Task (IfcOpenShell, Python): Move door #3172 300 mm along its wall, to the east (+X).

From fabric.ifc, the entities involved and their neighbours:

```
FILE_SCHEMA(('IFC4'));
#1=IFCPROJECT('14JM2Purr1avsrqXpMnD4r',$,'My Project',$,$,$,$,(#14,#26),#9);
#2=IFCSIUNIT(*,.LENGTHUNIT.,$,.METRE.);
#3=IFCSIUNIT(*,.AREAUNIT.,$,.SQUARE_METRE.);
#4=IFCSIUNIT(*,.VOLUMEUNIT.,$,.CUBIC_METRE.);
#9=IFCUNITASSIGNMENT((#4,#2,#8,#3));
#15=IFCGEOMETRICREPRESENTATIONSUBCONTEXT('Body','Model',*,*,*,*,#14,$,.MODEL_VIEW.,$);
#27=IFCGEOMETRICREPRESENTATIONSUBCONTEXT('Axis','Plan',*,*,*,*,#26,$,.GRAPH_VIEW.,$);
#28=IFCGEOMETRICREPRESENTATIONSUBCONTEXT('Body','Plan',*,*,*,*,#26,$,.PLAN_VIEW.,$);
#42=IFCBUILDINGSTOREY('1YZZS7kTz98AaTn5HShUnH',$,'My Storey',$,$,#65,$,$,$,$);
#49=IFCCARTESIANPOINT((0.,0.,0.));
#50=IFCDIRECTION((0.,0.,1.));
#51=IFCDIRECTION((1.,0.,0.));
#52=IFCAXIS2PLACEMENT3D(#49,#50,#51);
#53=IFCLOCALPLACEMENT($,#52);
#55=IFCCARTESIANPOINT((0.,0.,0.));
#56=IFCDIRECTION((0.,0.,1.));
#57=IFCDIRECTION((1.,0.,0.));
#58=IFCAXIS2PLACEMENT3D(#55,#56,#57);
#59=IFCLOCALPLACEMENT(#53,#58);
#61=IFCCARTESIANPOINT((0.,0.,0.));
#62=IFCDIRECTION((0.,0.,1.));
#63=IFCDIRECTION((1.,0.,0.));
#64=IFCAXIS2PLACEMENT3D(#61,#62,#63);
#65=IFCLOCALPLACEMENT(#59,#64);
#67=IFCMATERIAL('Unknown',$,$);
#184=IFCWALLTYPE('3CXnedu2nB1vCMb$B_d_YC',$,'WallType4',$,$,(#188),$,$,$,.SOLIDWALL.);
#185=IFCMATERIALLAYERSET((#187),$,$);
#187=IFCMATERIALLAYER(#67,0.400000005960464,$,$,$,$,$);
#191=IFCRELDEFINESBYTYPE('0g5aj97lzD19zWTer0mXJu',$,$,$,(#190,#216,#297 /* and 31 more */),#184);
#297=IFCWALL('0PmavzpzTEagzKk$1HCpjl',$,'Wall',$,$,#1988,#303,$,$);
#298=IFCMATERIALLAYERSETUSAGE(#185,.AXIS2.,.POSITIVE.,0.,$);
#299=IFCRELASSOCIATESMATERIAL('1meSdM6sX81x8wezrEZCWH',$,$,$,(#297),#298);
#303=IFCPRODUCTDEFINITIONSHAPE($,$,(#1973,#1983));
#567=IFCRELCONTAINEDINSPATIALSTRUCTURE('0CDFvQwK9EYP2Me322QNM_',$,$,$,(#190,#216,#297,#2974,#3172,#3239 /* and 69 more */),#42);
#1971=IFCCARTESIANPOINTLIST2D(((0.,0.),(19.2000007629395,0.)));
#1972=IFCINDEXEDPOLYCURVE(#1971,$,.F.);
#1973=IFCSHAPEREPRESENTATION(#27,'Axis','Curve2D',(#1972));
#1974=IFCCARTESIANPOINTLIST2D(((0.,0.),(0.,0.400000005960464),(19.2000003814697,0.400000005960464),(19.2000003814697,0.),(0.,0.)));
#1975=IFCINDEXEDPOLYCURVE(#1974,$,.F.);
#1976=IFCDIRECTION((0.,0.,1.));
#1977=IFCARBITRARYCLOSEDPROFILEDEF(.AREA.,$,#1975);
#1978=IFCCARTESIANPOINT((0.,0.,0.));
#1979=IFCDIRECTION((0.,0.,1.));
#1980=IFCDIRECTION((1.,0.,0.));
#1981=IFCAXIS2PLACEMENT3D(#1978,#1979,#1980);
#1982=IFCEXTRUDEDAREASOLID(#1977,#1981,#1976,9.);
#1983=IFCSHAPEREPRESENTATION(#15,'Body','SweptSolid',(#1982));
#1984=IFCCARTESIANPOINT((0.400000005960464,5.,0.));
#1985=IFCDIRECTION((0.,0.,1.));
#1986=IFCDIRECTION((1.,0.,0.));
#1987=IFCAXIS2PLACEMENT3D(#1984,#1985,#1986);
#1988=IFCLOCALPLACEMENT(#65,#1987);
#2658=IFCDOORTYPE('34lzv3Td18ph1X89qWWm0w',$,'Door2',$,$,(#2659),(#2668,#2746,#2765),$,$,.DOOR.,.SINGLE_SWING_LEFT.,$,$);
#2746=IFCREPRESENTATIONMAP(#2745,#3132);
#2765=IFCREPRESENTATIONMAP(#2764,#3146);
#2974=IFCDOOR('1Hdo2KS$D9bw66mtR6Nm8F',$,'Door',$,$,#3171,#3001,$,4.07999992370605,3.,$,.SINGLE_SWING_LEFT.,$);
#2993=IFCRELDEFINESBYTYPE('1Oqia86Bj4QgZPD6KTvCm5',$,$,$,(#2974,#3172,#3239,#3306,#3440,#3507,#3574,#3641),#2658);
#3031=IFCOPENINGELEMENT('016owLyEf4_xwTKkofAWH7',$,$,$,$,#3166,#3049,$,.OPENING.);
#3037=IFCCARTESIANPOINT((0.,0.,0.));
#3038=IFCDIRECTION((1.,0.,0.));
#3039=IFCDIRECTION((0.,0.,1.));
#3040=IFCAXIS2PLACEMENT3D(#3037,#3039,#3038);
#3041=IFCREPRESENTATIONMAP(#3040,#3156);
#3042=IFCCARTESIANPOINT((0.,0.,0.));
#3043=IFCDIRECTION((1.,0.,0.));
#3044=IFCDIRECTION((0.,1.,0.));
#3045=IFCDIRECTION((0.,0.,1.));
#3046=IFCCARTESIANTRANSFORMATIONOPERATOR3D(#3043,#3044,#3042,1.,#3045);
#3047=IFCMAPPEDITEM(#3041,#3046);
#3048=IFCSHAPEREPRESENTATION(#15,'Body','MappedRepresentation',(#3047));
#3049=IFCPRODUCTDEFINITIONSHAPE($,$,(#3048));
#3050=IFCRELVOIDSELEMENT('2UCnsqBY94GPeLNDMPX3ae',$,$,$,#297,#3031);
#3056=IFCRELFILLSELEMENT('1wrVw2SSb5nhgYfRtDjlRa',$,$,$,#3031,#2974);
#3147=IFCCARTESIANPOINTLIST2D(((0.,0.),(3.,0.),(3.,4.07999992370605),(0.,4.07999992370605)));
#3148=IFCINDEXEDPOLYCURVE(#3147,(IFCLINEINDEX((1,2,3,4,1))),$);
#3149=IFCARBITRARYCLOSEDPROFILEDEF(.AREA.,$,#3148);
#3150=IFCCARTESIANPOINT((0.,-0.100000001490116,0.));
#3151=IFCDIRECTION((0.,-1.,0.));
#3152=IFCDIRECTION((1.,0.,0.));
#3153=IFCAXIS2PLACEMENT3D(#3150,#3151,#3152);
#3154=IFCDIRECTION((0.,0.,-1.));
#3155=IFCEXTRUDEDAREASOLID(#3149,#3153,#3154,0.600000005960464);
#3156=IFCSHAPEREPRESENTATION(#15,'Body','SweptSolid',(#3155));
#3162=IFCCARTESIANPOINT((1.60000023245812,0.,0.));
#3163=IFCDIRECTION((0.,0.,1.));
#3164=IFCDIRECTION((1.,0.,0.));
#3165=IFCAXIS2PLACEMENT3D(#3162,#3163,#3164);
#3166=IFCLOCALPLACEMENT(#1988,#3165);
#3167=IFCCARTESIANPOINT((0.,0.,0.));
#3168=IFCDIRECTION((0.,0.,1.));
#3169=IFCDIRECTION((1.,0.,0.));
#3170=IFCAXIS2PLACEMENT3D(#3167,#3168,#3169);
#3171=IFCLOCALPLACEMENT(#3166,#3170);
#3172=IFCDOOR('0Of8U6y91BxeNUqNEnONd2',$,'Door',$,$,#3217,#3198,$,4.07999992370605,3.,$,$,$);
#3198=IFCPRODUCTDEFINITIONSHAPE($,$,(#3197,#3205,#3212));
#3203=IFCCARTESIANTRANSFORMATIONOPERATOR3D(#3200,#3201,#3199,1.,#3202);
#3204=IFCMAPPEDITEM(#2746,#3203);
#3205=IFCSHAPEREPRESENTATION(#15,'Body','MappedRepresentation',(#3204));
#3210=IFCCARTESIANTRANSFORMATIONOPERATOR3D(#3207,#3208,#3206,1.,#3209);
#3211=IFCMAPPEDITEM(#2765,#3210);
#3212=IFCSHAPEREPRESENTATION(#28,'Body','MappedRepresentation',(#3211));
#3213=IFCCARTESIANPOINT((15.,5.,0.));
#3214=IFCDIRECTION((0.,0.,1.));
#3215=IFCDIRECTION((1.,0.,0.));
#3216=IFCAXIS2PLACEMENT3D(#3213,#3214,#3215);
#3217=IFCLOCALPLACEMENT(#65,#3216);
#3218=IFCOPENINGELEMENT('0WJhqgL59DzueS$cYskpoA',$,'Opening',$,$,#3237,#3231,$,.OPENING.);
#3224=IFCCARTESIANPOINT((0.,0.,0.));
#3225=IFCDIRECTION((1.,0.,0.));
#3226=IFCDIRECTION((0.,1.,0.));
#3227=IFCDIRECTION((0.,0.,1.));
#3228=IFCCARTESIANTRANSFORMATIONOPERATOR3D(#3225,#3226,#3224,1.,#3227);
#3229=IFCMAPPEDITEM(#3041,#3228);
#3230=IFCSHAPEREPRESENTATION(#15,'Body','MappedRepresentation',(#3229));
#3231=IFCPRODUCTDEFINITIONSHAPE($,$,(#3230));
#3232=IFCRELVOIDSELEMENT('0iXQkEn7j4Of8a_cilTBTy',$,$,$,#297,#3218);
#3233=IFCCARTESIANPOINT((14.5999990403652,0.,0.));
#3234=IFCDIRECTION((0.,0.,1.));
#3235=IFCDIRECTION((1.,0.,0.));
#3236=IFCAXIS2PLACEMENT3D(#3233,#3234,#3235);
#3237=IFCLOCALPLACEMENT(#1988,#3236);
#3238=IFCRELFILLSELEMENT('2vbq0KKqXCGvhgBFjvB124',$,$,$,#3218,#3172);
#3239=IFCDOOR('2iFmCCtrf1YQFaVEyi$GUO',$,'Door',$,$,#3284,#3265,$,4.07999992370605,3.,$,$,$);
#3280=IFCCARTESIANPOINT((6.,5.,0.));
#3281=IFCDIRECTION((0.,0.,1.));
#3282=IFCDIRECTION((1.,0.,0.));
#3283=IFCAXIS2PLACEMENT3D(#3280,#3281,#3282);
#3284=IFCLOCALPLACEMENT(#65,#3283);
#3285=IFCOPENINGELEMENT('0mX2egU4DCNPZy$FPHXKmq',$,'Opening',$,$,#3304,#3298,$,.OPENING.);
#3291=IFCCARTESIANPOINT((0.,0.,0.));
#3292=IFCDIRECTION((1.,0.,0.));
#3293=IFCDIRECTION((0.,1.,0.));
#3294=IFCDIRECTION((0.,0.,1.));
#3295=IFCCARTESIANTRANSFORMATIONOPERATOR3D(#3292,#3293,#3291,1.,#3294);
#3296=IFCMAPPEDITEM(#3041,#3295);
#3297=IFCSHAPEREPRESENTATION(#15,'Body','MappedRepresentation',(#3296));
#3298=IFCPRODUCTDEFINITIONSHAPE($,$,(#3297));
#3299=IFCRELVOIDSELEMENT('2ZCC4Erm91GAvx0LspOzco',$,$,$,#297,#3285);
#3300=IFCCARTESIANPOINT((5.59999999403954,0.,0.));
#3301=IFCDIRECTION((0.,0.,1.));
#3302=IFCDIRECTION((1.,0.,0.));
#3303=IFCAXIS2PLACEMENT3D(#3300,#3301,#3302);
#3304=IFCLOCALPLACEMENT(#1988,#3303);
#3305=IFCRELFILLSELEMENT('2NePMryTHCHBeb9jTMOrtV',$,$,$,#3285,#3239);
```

```python
import ifcopenshell
import ifcopenshell.api.geometry
import ifcopenshell.util.placement
import ifcopenshell.util.unit

model = ifcopenshell.open("fabric.ifc")
unit_scale = ifcopenshell.util.unit.calculate_unit_scale(model)

door = model.by_id(3172)
opening = door.FillsVoids[0].RelatingOpeningElement
wall = opening.VoidsElements[0].RelatingBuildingElement

wall_matrix = ifcopenshell.util.placement.get_local_placement(wall.ObjectPlacement)
shift = wall_matrix[:3, 0] * 0.3 / unit_scale
before = ifcopenshell.util.placement.get_local_placement(door.ObjectPlacement)[:3, 3].copy()

# The door is not placed relative to its opening, so move both.
for product in (opening, door):
    matrix = ifcopenshell.util.placement.get_local_placement(product.ObjectPlacement)
    matrix[:3, 3] += shift
    ifcopenshell.api.geometry.edit_object_placement(model, product=product, matrix=matrix, is_si=False)

after = ifcopenshell.util.placement.get_local_placement(door.ObjectPlacement)[:3, 3]
print("door moved by", (after - before).round(3) + 0.0)

model.write("fabric-out.ifc")
```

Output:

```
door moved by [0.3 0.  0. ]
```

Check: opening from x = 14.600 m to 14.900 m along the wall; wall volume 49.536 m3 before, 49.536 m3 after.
